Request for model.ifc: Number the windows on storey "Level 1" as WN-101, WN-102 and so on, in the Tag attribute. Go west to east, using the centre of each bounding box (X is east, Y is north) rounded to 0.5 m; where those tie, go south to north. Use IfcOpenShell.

First a look at what the model holds.

```python
import ifcopenshell
import ifcopenshell.util.element
import ifcopenshell.util.placement

model = ifcopenshell.open("model.ifc")
print(model.schema)
storey = next(s for s in model.by_type("IfcBuildingStorey") if s.Name == "Level 1")
windows = [e for e in ifcopenshell.util.element.get_decomposition(storey) if e.is_a("IfcWindow")]
for e in sorted(windows, key=lambda e: e.id()):
    origin = ifcopenshell.util.placement.get_local_placement(e.ObjectPlacement)[:3, 3]
    print(e.id(), e.Tag, e.Name, origin.round(2) + 0.0, sep=" | ")
```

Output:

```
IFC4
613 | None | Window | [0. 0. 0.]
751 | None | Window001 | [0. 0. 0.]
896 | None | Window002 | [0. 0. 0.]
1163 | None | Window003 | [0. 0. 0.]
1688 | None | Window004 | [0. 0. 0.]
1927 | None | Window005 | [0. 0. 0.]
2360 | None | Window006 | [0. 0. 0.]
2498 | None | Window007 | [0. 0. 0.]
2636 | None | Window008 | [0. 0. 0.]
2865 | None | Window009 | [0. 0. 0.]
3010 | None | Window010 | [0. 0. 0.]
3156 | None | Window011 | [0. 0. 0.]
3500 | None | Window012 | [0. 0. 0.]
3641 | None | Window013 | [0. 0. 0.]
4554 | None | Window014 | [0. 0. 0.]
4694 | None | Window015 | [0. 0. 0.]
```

```python
import ifcopenshell
import ifcopenshell.geom
import ifcopenshell.util.element
import ifcopenshell.util.shape

model = ifcopenshell.open("model.ifc")
settings = ifcopenshell.geom.settings()
settings.set("use-world-coords", True)


def centre(element):
    shape = ifcopenshell.geom.create_shape(settings, element)
    return ifcopenshell.util.shape.get_bbox_centroid(shape.geometry)


storey = next(s for s in model.by_type("IfcBuildingStorey") if s.Name == "Level 1")
windows = [e for e in ifcopenshell.util.element.get_decomposition(storey) if e.is_a("IfcWindow")]

# Insertion points can sit at a corner or the storey origin, so sort by the geometry (in metres).
centres = {e: centre(e) for e in windows}
windows.sort(key=lambda e: (round(centres[e][0] / 0.5), centres[e][1]))

for i, e in enumerate(windows, start=1):
    number = f"WN-1{i:02d}"
    e.Tag = number
    print(e.id(), number)

model.write("model_edited.ifc")
```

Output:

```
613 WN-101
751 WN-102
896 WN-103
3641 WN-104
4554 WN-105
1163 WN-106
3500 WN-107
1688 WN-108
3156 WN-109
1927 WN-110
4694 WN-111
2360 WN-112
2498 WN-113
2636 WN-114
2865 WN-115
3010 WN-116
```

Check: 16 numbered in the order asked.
